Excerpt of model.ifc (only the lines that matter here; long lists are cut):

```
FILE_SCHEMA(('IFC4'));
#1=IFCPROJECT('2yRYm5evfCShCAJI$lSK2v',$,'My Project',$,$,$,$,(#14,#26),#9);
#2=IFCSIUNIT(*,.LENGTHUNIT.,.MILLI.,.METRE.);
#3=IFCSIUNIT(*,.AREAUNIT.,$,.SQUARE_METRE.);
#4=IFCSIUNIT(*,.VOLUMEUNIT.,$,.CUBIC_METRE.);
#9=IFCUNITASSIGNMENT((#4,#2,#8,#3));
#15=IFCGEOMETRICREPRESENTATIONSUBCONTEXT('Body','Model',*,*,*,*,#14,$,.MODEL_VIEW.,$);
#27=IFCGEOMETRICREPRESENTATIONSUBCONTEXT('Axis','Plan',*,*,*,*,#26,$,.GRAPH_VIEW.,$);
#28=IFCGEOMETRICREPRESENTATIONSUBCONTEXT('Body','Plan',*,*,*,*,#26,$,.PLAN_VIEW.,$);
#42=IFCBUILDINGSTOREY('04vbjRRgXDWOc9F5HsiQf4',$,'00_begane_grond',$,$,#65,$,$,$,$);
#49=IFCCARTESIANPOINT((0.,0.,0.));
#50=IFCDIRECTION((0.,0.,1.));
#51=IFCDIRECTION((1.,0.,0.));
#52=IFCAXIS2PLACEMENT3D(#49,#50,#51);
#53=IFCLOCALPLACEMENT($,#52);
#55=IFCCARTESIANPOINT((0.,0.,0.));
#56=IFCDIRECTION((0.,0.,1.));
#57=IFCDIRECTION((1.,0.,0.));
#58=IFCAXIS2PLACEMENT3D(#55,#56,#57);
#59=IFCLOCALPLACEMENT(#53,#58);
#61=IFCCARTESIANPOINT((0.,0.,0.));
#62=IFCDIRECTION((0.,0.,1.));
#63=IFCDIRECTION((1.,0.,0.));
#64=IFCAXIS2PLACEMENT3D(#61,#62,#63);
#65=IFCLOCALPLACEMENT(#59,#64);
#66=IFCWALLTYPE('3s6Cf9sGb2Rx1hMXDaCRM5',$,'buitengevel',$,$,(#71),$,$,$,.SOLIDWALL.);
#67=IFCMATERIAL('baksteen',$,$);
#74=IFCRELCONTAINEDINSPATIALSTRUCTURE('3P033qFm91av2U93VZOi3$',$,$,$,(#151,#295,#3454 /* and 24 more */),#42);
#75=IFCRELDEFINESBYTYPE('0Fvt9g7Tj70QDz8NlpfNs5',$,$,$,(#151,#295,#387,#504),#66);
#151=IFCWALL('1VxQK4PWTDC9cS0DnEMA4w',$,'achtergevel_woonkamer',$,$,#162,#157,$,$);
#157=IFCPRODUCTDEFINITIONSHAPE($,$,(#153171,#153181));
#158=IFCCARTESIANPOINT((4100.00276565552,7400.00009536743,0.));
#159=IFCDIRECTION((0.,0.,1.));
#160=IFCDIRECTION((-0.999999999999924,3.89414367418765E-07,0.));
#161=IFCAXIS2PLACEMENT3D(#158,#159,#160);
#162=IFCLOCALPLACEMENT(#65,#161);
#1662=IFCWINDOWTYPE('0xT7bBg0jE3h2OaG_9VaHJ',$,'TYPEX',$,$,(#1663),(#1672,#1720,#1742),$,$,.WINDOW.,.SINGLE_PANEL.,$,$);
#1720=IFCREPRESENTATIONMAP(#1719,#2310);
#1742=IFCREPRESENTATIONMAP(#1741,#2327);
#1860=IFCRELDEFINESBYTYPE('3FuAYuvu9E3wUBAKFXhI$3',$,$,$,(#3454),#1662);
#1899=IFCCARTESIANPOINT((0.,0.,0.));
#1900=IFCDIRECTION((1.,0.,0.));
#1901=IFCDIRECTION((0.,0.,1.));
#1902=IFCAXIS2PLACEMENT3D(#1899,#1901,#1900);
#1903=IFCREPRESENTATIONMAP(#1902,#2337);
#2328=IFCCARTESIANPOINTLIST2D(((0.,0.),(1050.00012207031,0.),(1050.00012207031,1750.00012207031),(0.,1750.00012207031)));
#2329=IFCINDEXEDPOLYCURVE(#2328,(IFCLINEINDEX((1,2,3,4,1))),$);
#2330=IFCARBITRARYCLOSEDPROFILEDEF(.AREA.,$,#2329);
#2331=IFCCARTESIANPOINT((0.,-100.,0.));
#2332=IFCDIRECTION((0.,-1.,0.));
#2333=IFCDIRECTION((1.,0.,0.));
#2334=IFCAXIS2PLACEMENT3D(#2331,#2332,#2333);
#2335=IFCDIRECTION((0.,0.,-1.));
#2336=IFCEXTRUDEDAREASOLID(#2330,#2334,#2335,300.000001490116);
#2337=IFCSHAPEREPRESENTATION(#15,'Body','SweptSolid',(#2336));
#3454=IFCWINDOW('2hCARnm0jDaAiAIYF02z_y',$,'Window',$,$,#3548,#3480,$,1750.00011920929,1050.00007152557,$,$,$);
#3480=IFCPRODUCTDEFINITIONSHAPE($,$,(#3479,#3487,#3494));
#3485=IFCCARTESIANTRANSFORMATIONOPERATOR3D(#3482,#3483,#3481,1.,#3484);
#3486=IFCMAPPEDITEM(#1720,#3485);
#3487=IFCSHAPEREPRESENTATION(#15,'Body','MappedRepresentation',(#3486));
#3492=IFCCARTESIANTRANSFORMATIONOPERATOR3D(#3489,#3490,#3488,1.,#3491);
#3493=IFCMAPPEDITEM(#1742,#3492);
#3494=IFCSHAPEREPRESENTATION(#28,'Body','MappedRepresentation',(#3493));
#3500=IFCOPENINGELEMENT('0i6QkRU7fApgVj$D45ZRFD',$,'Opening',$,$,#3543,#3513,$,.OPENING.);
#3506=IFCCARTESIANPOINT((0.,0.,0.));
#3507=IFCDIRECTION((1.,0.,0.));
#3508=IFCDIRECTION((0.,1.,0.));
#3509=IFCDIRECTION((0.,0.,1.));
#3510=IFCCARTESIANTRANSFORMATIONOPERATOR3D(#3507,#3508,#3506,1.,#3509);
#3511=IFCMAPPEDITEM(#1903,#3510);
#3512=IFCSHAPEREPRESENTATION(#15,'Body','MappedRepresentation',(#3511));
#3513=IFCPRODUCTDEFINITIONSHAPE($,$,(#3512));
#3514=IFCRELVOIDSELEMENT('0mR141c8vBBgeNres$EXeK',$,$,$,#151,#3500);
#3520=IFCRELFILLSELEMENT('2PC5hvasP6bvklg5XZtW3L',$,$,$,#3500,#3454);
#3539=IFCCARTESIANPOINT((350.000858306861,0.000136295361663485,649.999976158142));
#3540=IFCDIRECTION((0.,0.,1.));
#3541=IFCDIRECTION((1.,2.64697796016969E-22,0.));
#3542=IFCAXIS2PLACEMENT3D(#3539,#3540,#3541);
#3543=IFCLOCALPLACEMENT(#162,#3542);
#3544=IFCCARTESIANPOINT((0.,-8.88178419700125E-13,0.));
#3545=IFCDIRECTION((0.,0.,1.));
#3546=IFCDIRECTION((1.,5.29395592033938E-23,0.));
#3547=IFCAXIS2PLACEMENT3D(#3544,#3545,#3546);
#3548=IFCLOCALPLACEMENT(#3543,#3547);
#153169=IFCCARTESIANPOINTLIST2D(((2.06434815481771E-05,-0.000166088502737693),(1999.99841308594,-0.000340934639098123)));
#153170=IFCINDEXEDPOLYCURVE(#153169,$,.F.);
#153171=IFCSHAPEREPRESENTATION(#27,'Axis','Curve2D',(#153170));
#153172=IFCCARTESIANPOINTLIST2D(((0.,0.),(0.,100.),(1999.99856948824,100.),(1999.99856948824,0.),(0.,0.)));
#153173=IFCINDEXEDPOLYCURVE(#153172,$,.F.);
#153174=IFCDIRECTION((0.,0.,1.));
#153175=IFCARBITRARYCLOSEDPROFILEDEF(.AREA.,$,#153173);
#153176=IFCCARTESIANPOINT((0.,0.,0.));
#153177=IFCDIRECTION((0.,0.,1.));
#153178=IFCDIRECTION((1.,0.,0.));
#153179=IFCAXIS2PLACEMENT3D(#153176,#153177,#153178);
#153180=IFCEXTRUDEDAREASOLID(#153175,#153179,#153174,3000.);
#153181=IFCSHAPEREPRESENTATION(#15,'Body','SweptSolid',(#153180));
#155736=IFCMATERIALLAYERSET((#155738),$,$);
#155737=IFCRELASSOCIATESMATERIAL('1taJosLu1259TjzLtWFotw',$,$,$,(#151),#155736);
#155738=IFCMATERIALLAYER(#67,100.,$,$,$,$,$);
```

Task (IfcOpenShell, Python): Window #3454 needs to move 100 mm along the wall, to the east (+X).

```python
import ifcopenshell
import ifcopenshell.api.geometry
import ifcopenshell.util.placement

model = ifcopenshell.open("model.ifc")

window = model.by_id(3454)
opening = window.FillsVoids[0].RelatingOpeningElement
wall = opening.VoidsElements[0].RelatingBuildingElement

wall_matrix = ifcopenshell.util.placement.get_local_placement(wall.ObjectPlacement)
shift = wall_matrix[:3, 0] * -100.0
before = ifcopenshell.util.placement.get_local_placement(window.ObjectPlacement)[:3, 3].copy()

# The window is placed relative to its opening, so it follows when the opening moves.
matrix = ifcopenshell.util.placement.get_local_placement(opening.ObjectPlacement)
matrix[:3, 3] += shift
ifcopenshell.api.geometry.edit_object_placement(
    model, product=opening, matrix=matrix, is_si=False, should_transform_children=True
)

after = ifcopenshell.util.placement.get_local_placement(window.ObjectPlacement)[:3, 3]
print("window moved by", (after - before).round(3) + 0.0)

model.write("model_rev.ifc")
```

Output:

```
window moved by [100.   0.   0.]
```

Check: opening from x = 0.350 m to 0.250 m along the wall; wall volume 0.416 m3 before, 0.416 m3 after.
